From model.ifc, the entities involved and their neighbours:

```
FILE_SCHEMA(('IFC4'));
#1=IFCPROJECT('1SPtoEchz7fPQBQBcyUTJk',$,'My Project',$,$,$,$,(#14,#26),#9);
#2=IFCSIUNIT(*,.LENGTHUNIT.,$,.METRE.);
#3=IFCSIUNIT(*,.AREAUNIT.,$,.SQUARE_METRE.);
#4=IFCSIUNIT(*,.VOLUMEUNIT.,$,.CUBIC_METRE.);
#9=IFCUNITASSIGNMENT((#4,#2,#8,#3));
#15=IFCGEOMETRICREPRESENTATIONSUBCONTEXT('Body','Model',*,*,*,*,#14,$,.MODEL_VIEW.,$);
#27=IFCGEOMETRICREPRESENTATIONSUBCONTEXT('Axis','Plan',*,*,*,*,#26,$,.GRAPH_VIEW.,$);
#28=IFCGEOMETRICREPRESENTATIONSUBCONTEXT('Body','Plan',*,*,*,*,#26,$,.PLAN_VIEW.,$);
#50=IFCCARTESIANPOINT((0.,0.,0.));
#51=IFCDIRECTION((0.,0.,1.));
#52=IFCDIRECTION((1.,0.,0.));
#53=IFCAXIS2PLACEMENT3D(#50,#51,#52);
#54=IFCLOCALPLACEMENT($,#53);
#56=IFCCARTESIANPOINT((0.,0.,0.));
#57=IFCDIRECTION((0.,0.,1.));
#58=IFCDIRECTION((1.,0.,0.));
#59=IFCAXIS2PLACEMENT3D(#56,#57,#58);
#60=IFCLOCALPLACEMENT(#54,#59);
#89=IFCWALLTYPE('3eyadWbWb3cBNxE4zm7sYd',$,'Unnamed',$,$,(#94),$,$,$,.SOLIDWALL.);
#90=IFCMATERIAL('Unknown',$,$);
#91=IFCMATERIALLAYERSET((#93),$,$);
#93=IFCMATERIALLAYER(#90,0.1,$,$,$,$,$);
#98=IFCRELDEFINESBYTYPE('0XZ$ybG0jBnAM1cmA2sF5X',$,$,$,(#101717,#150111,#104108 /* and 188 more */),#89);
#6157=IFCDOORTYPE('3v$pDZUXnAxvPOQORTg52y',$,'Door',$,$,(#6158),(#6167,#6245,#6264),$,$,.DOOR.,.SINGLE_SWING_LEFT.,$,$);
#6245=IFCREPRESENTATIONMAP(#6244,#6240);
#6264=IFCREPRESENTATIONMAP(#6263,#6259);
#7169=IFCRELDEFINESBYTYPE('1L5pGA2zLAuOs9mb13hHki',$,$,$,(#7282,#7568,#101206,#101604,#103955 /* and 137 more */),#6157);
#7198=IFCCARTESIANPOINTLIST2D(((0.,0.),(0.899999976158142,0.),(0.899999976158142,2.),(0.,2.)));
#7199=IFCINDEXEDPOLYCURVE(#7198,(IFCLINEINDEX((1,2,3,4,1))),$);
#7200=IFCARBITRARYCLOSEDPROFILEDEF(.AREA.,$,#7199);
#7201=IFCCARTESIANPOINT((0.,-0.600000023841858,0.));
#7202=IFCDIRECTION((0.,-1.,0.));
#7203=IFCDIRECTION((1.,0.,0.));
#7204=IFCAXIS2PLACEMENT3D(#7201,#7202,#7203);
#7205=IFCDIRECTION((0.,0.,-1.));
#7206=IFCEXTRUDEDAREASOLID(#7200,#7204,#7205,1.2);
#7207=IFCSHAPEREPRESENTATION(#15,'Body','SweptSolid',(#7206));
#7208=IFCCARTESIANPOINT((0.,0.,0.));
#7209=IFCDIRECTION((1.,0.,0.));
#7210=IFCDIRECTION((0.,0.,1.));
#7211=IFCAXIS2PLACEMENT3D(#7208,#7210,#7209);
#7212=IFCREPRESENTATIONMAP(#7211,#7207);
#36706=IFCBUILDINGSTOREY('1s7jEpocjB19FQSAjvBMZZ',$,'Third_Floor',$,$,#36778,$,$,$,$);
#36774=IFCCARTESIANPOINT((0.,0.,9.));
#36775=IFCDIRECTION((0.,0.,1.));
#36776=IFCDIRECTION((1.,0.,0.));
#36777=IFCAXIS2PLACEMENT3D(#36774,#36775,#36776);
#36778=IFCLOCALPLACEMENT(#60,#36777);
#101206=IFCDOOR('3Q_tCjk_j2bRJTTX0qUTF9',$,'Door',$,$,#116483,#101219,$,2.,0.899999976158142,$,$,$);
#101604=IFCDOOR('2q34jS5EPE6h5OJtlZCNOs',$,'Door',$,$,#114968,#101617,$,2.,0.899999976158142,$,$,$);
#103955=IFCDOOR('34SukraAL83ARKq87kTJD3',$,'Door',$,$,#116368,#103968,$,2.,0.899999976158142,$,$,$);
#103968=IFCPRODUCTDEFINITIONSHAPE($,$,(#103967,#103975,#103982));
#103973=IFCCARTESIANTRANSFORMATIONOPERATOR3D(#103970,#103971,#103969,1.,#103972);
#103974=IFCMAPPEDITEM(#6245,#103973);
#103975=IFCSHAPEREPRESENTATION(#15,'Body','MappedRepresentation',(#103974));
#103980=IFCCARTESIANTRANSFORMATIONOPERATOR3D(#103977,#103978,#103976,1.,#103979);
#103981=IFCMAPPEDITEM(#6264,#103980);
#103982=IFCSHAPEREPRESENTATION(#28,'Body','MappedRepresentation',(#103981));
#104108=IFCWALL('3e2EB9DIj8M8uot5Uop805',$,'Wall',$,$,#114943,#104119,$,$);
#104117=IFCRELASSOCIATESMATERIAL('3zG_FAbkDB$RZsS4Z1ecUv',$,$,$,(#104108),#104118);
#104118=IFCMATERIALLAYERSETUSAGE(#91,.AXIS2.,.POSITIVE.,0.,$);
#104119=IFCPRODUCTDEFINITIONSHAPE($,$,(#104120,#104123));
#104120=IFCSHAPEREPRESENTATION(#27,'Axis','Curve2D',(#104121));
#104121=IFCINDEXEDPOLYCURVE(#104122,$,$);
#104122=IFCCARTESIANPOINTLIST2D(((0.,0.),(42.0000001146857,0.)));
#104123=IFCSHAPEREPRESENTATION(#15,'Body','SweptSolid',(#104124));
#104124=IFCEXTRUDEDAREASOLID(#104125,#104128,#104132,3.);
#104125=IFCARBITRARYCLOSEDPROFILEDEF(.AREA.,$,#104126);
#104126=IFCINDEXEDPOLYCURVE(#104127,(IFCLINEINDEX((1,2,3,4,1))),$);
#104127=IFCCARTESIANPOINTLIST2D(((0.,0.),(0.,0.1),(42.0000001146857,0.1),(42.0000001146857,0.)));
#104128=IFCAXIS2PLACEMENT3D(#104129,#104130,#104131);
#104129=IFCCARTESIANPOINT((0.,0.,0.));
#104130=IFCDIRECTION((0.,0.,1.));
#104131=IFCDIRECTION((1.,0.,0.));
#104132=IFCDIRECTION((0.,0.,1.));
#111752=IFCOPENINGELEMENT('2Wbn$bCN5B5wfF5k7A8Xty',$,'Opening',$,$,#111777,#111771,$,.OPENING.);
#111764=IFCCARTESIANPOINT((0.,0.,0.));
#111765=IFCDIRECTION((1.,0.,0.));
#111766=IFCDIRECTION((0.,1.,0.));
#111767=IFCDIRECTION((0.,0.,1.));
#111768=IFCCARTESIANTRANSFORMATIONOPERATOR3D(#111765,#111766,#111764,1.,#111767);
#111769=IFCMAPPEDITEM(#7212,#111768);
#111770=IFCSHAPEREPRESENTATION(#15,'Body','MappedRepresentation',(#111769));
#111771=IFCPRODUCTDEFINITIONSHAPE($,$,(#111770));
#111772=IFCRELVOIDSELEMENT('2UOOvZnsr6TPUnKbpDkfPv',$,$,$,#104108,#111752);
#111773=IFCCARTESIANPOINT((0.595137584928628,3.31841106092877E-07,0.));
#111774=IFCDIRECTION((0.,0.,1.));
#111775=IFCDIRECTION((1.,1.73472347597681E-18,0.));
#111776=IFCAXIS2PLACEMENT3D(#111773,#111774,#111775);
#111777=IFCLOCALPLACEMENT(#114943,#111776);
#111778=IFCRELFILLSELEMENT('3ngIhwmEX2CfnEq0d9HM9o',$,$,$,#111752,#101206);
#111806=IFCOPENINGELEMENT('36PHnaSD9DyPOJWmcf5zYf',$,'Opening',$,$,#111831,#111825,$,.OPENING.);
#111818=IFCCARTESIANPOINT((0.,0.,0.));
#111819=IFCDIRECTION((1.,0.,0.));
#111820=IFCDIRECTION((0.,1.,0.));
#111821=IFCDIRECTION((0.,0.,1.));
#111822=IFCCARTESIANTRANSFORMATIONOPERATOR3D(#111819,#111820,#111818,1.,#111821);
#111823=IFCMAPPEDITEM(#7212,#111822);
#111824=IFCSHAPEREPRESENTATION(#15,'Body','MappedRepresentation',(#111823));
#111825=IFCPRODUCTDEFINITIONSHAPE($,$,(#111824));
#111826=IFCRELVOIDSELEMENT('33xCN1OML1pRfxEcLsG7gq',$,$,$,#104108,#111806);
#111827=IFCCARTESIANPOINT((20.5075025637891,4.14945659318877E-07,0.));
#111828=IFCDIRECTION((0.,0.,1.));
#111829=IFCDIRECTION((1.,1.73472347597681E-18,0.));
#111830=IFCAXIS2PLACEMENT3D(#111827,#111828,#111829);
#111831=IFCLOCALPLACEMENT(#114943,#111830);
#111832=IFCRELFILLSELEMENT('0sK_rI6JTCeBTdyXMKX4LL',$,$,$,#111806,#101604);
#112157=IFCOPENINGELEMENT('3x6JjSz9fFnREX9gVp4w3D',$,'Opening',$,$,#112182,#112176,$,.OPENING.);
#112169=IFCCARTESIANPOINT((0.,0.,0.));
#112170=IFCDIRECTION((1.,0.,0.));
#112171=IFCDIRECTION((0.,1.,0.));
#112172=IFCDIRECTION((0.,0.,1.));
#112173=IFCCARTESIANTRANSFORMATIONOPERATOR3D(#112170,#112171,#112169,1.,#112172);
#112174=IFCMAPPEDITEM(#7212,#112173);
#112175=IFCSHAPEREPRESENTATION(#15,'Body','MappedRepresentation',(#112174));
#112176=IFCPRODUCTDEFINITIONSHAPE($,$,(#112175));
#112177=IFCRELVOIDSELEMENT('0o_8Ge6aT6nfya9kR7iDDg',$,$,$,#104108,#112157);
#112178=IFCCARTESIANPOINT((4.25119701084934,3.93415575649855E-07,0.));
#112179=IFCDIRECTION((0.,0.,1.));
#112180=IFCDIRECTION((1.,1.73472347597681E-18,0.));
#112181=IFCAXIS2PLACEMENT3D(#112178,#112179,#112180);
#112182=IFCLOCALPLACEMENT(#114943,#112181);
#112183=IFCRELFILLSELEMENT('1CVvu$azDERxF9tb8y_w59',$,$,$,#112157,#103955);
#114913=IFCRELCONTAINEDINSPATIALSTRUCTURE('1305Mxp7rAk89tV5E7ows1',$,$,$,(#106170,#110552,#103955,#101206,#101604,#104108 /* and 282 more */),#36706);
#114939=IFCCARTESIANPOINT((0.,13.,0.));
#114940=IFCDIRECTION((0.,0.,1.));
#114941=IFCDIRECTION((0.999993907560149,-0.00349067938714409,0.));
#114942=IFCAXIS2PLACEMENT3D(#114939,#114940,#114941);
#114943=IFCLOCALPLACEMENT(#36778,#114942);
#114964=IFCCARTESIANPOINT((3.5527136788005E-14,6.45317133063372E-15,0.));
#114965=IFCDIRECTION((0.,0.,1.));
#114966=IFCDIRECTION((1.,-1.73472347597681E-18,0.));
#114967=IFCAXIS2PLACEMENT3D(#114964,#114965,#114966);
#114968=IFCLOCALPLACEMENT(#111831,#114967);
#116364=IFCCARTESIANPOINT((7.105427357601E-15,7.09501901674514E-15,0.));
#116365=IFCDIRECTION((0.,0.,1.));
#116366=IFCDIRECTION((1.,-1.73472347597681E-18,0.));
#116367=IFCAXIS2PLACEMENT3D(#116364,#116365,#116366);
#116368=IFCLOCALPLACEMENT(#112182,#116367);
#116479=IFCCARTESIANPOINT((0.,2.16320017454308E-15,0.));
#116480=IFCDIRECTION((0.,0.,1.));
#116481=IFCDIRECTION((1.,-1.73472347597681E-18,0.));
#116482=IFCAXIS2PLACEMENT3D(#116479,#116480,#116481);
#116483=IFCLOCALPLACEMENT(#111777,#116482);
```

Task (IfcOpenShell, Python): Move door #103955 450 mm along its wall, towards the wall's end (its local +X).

```python
import ifcopenshell
import ifcopenshell.api.geometry
import ifcopenshell.util.placement
import ifcopenshell.util.unit

model = ifcopenshell.open("model.ifc")
unit_scale = ifcopenshell.util.unit.calculate_unit_scale(model)

door = model.by_guid("34SukraAL83ARKq87kTJD3")
opening = door.FillsVoids[0].RelatingOpeningElement
wall = opening.VoidsElements[0].RelatingBuildingElement

wall_matrix = ifcopenshell.util.placement.get_local_placement(wall.ObjectPlacement)
shift = wall_matrix[:3, 0] * 0.45 / unit_scale
before = ifcopenshell.util.placement.get_local_placement(door.ObjectPlacement)[:3, 3].copy()

# The door is placed relative to its opening, so it follows when the opening moves.
matrix = ifcopenshell.util.placement.get_local_placement(opening.ObjectPlacement)
matrix[:3, 3] += shift
ifcopenshell.api.geometry.edit_object_placement(
    model, product=opening, matrix=matrix, is_si=False, should_transform_children=True
)

after = ifcopenshell.util.placement.get_local_placement(door.ObjectPlacement)[:3, 3]
print("door moved by", (after - before).round(3) + 0.0)

model.write("model_v2.ifc")
```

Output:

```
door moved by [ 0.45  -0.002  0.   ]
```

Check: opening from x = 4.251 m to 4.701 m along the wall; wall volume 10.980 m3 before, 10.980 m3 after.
